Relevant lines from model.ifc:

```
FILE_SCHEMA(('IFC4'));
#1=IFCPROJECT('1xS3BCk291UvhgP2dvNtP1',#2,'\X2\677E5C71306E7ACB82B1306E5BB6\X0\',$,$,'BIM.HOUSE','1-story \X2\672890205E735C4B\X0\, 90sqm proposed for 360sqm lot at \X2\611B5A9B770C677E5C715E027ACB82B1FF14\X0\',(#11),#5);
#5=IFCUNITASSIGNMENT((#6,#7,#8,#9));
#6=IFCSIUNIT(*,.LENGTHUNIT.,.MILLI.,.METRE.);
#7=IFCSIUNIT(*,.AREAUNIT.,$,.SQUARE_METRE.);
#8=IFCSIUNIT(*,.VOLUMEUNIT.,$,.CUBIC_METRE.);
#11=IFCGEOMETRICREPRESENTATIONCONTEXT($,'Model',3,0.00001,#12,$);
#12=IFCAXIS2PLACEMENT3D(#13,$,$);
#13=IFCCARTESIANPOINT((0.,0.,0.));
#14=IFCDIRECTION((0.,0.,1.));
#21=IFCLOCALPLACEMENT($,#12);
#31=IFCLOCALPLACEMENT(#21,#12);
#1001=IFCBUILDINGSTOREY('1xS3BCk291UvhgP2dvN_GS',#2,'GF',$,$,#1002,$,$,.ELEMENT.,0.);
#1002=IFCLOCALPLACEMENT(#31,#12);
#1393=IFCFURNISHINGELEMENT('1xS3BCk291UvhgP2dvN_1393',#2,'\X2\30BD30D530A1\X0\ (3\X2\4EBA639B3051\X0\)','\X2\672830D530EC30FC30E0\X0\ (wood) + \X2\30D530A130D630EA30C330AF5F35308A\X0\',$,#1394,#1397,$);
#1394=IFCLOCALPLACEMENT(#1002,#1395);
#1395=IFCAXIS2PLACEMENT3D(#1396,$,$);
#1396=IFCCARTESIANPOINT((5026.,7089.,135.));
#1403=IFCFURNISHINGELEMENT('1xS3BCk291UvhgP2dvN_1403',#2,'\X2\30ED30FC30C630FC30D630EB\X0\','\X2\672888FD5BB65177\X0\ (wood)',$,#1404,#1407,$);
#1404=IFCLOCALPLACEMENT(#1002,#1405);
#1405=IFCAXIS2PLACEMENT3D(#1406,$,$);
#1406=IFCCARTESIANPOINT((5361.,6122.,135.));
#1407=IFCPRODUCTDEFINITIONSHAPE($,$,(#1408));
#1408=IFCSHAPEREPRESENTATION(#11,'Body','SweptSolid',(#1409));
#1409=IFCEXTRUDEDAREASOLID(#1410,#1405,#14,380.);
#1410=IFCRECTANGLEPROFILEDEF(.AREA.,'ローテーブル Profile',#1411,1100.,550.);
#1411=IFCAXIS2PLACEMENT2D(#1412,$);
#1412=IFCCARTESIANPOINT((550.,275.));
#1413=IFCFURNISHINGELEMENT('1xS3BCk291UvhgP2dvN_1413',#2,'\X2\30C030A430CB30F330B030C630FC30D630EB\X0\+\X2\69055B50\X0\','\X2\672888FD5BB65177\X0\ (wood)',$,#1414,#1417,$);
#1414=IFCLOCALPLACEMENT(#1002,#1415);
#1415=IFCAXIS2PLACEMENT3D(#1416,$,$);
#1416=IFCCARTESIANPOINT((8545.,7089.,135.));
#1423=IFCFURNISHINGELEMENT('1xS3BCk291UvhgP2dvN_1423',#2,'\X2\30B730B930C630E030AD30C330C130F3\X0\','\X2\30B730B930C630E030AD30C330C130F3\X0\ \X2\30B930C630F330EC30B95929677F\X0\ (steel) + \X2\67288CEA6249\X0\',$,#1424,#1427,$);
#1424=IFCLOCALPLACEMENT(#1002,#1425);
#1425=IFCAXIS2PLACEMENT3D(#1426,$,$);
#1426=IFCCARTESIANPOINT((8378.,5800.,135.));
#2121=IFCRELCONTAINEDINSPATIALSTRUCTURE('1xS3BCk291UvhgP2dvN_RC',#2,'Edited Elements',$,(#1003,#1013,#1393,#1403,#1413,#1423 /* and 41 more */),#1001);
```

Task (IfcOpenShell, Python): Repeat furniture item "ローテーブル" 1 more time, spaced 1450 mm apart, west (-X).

```python
import numpy as np
import ifcopenshell
import ifcopenshell.api.geometry
import ifcopenshell.api.root
import ifcopenshell.util.element
import ifcopenshell.util.placement
import ifcopenshell.util.unit

model = ifcopenshell.open("model.ifc")
unit_scale = ifcopenshell.util.unit.calculate_unit_scale(model)


def reuse_history(source, copy):
    """copy_class also copies each property set's owner history, people and application; keep the originals."""
    for rel in copy.IsDefinedBy:
        if rel.is_a("IfcRelDefinesByProperties") and (history := rel.RelatingPropertyDefinition.OwnerHistory):
            rel.RelatingPropertyDefinition.OwnerHistory = source.OwnerHistory
            ifcopenshell.util.element.remove_deep2(model, history)


source = model.by_id(1403)
base = ifcopenshell.util.placement.get_local_placement(source.ObjectPlacement)
step = np.array([-1.0, 0.0, 0.0]) * 1.45 / unit_scale

for i in range(1, 2):
    copy = ifcopenshell.api.root.copy_class(model, product=source)
    copy.Representation = ifcopenshell.util.element.copy_deep(
        model, source.Representation, exclude=["IfcGeometricRepresentationContext", "IfcRepresentationMap"]
    )
    reuse_history(source, copy)
    matrix = base.copy()
    matrix[:3, 3] += i * step
    print("added at", matrix[:3, 3].round(3) + 0.0)
    ifcopenshell.api.geometry.edit_object_placement(model, product=copy, matrix=matrix, is_si=False)

model.write("model_edited.ifc")
```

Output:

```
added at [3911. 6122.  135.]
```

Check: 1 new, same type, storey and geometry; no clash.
